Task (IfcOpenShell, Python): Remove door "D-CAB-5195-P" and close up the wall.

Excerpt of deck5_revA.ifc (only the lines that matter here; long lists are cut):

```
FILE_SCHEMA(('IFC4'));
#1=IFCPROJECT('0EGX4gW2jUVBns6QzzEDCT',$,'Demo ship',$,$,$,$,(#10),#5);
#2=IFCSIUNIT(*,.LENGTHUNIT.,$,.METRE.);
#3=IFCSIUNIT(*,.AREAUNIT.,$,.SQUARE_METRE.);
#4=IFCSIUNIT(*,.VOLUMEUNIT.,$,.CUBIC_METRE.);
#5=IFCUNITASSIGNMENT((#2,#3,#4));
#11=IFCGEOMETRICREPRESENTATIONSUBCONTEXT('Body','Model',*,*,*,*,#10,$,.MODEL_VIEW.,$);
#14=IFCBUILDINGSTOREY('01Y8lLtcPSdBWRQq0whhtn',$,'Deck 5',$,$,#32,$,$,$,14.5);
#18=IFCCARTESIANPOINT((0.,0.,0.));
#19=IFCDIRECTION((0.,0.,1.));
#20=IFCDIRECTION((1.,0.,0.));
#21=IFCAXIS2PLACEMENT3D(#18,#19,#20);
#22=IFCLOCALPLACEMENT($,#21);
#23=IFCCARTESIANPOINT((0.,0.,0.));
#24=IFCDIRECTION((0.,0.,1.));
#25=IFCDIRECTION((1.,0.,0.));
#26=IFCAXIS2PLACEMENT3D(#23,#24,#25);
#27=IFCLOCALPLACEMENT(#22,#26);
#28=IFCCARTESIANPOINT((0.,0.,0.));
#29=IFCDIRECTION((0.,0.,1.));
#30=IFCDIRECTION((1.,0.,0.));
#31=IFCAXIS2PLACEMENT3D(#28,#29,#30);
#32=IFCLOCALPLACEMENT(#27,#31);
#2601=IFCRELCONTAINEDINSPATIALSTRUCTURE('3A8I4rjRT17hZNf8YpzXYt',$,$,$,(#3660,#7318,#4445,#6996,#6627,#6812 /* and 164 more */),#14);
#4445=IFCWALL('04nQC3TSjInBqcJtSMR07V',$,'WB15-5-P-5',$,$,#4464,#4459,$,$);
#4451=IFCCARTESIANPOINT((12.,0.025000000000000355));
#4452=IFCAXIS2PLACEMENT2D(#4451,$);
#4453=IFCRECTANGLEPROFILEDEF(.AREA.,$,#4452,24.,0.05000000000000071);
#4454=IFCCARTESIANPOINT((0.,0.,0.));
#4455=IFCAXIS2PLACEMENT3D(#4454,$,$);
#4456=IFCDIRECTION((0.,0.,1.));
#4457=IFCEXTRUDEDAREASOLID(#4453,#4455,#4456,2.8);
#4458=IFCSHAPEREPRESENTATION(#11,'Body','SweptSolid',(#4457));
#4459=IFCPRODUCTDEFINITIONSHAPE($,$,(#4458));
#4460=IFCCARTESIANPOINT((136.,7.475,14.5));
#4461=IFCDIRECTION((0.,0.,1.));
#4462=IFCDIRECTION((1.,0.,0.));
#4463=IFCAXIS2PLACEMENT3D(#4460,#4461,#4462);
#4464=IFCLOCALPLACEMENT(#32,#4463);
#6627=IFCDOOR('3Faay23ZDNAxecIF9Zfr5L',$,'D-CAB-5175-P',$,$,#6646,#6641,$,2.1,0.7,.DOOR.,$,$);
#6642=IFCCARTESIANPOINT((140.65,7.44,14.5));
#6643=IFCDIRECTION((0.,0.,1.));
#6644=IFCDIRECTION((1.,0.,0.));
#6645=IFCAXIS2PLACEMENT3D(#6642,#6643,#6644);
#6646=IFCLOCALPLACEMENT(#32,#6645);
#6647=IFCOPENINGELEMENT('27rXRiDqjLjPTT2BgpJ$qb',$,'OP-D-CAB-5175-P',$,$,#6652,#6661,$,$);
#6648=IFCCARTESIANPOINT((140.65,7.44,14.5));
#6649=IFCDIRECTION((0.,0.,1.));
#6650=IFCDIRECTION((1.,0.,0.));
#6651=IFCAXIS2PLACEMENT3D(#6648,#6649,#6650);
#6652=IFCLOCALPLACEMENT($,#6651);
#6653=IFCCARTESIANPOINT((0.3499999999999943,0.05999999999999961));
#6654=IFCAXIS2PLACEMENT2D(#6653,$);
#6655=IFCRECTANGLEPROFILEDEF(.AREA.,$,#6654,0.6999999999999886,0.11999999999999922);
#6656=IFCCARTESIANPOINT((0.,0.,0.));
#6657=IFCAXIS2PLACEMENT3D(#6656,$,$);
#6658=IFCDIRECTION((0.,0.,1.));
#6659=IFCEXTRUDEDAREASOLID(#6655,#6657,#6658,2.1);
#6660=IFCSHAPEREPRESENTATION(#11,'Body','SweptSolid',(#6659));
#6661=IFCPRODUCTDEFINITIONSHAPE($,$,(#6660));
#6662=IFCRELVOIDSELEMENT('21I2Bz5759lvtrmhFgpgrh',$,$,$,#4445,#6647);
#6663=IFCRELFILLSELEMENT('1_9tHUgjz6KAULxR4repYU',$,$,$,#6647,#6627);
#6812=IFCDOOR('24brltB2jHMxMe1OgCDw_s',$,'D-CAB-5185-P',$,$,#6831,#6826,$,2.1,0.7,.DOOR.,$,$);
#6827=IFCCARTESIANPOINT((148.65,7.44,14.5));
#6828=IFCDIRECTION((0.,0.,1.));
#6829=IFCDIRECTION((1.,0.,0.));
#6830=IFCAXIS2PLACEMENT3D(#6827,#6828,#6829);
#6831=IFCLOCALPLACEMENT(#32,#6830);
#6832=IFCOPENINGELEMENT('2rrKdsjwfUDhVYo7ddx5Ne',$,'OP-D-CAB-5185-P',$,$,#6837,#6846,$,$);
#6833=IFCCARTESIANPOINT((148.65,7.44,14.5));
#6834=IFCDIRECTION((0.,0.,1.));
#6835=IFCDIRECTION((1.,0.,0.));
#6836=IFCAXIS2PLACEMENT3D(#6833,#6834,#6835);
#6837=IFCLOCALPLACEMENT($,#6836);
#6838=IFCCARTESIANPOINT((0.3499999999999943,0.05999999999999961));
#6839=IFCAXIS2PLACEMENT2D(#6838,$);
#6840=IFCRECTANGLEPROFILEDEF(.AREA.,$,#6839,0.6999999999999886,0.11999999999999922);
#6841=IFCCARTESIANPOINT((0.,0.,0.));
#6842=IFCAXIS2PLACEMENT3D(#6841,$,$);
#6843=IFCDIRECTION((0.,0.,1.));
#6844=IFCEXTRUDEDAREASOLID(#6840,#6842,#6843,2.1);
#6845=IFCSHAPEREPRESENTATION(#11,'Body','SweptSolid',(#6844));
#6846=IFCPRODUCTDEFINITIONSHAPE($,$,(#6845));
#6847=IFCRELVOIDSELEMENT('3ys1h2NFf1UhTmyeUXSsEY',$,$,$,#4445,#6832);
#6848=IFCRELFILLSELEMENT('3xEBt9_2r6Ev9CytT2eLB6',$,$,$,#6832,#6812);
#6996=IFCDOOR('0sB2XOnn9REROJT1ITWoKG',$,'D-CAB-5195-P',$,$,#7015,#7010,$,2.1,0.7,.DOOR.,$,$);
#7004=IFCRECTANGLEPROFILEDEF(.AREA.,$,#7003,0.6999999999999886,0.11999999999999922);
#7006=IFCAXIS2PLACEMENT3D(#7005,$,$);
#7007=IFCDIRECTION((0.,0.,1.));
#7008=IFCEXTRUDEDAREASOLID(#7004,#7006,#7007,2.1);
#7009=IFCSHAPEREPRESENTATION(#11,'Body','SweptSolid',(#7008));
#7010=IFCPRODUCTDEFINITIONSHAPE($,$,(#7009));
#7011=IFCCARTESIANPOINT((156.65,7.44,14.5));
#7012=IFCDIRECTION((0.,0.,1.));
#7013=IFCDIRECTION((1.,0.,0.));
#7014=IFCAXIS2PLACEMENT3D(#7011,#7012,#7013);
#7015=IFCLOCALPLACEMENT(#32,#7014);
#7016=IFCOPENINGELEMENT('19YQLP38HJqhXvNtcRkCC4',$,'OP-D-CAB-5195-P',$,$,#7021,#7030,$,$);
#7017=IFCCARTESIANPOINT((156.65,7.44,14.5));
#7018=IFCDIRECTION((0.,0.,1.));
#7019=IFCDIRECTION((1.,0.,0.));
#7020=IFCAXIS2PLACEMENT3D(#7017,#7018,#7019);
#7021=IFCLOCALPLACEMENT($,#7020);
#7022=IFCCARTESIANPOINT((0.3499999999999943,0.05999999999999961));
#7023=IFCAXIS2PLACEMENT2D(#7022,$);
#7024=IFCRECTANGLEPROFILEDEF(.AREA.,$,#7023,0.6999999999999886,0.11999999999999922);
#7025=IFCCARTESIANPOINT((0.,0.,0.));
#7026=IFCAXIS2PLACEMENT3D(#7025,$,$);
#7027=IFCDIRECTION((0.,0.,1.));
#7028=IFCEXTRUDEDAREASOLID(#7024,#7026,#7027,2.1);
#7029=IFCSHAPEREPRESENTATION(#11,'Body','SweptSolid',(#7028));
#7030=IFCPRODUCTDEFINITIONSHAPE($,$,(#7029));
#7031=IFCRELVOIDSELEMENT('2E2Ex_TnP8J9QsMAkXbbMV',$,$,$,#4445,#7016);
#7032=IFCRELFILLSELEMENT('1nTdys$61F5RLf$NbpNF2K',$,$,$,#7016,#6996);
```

```python
import ifcopenshell
import ifcopenshell.api.feature
import ifcopenshell.api.root
import ifcopenshell.geom
import ifcopenshell.util.shape

model = ifcopenshell.open("deck5_revA.ifc")
settings = ifcopenshell.geom.settings()


def volume(element):
    """Net volume in cubic metres, openings subtracted."""
    shape = ifcopenshell.geom.create_shape(settings, element)
    return ifcopenshell.util.shape.get_volume(shape.geometry)


door = model.by_guid("0sB2XOnn9REROJT1ITWoKG")
opening = door.FillsVoids[0].RelatingOpeningElement
wall = opening.VoidsElements[0].RelatingBuildingElement
before = volume(wall)

ifcopenshell.api.root.remove_product(model, product=door)
ifcopenshell.api.feature.remove_feature(model, feature=opening)

after = volume(wall)

print(f"wall volume {before:.3f} -> {after:.3f} m3")

model.write("deck5_revA_rev.ifc")
```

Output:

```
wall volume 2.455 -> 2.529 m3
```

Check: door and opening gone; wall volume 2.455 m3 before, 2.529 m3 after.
